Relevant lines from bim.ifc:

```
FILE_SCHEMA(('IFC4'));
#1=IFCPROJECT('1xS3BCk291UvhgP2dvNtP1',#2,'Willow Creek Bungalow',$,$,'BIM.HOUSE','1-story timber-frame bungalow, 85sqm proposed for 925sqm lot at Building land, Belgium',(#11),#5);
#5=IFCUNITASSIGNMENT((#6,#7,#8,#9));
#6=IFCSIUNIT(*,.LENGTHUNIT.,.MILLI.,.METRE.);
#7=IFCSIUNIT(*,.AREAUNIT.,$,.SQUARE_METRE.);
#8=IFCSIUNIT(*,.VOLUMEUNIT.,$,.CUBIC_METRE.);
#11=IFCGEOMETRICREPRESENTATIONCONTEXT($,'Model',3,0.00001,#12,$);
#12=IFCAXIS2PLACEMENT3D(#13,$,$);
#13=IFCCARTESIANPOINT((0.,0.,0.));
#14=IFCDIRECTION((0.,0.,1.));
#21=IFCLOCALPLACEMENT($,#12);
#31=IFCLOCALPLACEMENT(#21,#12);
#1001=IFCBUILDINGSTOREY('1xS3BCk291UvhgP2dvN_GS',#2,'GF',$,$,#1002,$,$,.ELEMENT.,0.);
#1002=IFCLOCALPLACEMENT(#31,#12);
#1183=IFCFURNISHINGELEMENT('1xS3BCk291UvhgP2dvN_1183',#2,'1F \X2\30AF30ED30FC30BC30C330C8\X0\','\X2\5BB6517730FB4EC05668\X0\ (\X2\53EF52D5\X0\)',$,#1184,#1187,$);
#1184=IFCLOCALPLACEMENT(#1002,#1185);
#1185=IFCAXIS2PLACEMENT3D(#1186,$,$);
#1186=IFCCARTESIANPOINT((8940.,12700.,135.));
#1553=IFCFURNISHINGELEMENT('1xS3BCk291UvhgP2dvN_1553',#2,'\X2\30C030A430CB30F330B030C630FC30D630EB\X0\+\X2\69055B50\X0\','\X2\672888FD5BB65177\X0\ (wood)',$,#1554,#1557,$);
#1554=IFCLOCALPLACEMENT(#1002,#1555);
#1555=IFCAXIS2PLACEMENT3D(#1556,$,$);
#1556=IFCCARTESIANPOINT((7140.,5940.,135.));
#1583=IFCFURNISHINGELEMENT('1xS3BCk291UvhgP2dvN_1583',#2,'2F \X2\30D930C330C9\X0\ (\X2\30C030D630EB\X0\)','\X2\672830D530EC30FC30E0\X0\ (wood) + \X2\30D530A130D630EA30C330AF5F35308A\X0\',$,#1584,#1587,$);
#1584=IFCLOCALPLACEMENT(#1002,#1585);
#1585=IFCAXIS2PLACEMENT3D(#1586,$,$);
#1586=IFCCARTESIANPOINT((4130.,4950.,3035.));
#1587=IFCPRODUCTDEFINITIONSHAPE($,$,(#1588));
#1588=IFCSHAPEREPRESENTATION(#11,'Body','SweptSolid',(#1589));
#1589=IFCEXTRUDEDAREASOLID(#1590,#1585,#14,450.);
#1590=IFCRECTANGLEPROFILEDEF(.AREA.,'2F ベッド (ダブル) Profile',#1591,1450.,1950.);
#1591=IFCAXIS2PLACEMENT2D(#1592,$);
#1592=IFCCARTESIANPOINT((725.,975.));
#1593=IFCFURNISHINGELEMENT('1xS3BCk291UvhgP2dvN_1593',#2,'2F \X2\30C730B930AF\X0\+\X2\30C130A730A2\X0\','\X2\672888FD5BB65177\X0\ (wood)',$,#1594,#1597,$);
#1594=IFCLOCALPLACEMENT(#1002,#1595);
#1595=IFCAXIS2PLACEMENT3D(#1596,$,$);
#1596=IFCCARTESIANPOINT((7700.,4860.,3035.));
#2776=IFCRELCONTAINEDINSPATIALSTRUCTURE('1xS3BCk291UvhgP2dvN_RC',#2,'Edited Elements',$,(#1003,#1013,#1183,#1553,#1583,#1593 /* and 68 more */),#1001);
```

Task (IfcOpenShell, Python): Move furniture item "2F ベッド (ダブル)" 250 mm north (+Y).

```python
import ifcopenshell
import ifcopenshell.api.geometry
import ifcopenshell.util.placement

model = ifcopenshell.open("bim.ifc")

item = model.by_guid("1xS3BCk291UvhgP2dvN_1583")
matrix = ifcopenshell.util.placement.get_local_placement(item.ObjectPlacement)
matrix[1, 3] += 250.0
ifcopenshell.api.geometry.edit_object_placement(model, product=item, matrix=matrix, is_si=False)

print(ifcopenshell.util.placement.get_local_placement(item.ObjectPlacement).round(3) + 0.0)

model.write("bim_rev.ifc")
```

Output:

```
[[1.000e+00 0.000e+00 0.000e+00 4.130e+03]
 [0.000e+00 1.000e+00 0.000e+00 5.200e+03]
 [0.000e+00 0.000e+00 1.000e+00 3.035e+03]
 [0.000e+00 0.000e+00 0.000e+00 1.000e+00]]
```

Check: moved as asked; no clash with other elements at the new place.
